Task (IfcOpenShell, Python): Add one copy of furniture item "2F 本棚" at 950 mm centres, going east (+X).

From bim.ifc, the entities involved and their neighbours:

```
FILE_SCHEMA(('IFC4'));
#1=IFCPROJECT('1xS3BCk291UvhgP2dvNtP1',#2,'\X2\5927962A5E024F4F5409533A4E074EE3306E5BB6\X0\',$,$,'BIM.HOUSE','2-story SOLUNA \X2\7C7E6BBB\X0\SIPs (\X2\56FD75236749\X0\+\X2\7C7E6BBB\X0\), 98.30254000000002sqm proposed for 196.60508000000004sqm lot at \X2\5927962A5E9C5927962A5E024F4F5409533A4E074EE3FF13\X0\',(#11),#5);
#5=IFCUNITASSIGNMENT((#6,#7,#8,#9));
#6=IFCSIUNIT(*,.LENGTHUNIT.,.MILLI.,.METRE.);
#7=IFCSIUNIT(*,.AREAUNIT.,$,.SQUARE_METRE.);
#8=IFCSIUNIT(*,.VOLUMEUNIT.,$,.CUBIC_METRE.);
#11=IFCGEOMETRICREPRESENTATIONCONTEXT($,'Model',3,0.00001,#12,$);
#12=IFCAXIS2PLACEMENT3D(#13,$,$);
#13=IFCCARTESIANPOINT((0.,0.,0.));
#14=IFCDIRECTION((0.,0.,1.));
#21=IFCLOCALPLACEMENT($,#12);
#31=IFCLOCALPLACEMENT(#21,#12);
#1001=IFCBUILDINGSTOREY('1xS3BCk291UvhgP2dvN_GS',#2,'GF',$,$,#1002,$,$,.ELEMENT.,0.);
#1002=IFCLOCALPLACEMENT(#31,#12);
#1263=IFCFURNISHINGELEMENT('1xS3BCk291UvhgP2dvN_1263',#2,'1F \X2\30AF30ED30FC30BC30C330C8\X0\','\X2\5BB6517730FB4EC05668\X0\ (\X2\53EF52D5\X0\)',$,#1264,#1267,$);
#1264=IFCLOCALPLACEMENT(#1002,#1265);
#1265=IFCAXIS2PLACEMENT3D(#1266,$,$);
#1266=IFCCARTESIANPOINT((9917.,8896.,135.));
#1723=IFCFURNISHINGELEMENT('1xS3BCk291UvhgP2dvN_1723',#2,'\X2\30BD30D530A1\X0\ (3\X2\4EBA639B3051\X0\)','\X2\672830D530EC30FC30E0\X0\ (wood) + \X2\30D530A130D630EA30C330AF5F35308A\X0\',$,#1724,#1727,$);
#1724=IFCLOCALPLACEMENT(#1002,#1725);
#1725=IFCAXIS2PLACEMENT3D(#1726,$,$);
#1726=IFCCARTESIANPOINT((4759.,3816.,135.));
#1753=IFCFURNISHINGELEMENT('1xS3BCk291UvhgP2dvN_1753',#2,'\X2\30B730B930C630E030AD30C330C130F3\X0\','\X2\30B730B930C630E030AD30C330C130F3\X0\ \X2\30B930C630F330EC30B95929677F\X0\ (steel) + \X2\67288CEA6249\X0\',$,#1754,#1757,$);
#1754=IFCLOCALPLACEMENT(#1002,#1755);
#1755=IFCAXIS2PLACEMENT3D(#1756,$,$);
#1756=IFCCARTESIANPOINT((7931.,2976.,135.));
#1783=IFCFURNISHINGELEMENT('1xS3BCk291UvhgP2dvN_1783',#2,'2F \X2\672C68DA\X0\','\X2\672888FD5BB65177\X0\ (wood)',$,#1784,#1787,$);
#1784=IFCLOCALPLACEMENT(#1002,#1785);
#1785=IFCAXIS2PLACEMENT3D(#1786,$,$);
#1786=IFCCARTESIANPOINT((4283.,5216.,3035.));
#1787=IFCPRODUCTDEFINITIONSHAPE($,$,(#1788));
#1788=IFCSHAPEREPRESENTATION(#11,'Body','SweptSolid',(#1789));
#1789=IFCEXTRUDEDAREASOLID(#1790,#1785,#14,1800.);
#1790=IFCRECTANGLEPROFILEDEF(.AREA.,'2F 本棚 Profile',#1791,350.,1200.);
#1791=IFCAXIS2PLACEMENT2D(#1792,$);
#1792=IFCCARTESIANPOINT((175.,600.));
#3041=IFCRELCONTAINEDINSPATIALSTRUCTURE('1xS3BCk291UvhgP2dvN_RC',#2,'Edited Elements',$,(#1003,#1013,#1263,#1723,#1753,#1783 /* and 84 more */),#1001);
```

```python
import numpy as np
import ifcopenshell
import ifcopenshell.api.geometry
import ifcopenshell.api.root
import ifcopenshell.util.element
import ifcopenshell.util.placement
import ifcopenshell.util.unit

model = ifcopenshell.open("bim.ifc")
unit_scale = ifcopenshell.util.unit.calculate_unit_scale(model)


def reuse_history(source, copy):
    """copy_class also copies each property set's owner history, people and application; keep the originals."""
    for rel in copy.IsDefinedBy:
        if rel.is_a("IfcRelDefinesByProperties") and (history := rel.RelatingPropertyDefinition.OwnerHistory):
            rel.RelatingPropertyDefinition.OwnerHistory = source.OwnerHistory
            ifcopenshell.util.element.remove_deep2(model, history)


source = model.by_guid("1xS3BCk291UvhgP2dvN_1783")
base = ifcopenshell.util.placement.get_local_placement(source.ObjectPlacement)
step = np.array([1.0, 0.0, 0.0]) * 0.95 / unit_scale

for i in range(1, 2):
    copy = ifcopenshell.api.root.copy_class(model, product=source)
    copy.Representation = ifcopenshell.util.element.copy_deep(
        model, source.Representation, exclude=["IfcGeometricRepresentationContext", "IfcRepresentationMap"]
    )
    reuse_history(source, copy)
    matrix = base.copy()
    matrix[:3, 3] += i * step
    print("added at", matrix[:3, 3].round(3) + 0.0)
    ifcopenshell.api.geometry.edit_object_placement(model, product=copy, matrix=matrix, is_si=False)

model.write("bim_updated.ifc")
```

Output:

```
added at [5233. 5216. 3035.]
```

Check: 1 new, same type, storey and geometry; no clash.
